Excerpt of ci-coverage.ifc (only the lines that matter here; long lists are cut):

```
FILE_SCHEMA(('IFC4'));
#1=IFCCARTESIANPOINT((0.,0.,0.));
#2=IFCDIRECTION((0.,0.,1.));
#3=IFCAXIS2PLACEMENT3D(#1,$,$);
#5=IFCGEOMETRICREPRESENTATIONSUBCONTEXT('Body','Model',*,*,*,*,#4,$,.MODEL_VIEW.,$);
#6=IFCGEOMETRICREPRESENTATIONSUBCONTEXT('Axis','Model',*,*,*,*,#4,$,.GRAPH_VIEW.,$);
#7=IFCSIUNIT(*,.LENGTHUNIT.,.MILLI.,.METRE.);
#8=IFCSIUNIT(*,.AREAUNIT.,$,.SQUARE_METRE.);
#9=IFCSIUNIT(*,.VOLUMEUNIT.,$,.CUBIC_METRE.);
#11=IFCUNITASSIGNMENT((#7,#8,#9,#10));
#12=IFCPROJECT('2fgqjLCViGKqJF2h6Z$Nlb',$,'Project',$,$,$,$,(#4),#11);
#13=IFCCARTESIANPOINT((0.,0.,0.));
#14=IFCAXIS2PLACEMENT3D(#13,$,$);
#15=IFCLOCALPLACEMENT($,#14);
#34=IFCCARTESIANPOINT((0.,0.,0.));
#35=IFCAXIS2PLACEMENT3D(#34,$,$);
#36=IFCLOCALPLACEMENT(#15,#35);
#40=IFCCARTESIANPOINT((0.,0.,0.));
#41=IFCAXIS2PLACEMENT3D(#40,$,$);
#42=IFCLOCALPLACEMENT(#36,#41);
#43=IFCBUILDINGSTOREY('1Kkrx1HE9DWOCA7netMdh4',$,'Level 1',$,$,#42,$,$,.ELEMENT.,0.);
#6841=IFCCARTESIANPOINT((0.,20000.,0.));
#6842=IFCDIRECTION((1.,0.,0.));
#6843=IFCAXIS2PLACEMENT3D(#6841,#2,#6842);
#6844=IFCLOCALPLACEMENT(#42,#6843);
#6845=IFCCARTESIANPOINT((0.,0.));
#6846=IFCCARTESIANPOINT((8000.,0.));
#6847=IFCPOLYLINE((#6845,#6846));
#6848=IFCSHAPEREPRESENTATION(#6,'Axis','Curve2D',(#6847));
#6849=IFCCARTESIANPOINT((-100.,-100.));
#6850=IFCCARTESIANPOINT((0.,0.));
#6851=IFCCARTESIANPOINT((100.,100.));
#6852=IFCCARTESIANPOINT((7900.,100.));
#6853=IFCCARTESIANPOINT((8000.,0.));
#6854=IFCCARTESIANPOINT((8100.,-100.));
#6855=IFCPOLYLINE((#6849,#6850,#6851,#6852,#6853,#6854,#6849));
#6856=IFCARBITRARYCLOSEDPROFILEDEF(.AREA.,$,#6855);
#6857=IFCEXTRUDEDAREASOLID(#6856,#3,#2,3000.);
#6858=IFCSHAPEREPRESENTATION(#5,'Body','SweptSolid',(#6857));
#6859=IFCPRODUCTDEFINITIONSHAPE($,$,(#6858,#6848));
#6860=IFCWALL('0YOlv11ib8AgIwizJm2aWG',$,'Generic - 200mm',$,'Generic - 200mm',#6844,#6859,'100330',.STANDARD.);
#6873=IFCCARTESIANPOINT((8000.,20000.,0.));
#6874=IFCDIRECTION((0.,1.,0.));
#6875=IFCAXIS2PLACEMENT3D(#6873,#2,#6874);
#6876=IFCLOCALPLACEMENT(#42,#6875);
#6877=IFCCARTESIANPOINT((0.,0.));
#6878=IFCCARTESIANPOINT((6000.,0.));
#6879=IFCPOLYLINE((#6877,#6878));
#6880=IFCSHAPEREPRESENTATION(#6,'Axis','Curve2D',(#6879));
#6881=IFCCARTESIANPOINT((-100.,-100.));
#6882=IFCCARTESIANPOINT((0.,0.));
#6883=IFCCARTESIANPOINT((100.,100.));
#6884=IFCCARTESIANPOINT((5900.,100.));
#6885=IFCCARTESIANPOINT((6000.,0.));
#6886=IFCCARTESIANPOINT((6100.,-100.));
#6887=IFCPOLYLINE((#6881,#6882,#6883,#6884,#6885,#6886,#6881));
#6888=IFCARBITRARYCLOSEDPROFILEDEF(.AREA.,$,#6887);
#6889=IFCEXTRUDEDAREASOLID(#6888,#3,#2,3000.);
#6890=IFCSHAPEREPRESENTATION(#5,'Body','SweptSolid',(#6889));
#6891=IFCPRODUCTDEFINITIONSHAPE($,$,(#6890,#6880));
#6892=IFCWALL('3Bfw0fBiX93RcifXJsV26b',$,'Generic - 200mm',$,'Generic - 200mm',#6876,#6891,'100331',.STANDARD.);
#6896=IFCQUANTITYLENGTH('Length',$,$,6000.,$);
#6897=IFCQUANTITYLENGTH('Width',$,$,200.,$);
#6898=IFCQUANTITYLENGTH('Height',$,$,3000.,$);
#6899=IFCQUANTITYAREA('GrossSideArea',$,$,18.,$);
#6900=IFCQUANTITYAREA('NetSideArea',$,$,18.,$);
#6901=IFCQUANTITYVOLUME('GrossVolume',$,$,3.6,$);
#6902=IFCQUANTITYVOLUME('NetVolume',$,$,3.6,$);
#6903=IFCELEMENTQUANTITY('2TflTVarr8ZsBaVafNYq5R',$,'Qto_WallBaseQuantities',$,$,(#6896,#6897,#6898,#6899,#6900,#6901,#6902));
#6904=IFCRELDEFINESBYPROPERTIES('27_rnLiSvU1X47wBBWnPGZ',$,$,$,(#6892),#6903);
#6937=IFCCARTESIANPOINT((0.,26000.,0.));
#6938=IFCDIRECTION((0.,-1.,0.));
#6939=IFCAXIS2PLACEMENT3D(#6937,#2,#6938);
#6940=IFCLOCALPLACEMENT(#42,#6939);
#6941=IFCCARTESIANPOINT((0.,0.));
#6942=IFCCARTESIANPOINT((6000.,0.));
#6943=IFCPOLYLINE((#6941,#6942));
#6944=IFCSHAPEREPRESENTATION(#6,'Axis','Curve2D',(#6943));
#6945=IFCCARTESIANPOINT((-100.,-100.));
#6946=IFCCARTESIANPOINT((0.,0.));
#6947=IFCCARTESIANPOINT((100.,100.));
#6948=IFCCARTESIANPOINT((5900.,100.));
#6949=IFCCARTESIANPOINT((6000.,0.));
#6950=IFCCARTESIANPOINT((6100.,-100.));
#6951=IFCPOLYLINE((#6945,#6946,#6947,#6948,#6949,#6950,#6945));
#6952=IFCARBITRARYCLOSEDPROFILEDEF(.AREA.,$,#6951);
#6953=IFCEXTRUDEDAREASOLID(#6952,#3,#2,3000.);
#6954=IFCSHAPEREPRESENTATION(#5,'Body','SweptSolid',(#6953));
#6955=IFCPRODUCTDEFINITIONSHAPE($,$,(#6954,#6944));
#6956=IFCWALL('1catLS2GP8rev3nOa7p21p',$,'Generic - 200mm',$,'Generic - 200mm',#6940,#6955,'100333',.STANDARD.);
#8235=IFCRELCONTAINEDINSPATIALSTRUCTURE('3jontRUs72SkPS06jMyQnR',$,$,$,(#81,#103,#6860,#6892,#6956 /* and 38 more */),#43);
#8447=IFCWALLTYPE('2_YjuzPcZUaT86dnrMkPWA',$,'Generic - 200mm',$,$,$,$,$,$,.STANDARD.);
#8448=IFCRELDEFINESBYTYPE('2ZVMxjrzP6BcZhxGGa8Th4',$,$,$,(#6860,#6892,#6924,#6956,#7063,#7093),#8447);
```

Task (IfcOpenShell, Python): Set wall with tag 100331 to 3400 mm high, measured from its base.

```python
import ifcopenshell
import ifcopenshell.api.pset
import ifcopenshell.geom
import ifcopenshell.util.element
import ifcopenshell.util.representation
import ifcopenshell.util.shape
import ifcopenshell.util.unit

model = ifcopenshell.open("ci-coverage.ifc")
unit_scale = ifcopenshell.util.unit.calculate_unit_scale(model)
area_scale = ifcopenshell.util.unit.calculate_unit_scale(model, "AREAUNIT")
volume_scale = ifcopenshell.util.unit.calculate_unit_scale(model, "VOLUMEUNIT")
settings = ifcopenshell.geom.settings()


def volume(element):
    """Net volume in cubic metres, openings subtracted."""
    shape = ifcopenshell.geom.create_shape(settings, element)
    return ifcopenshell.util.shape.get_volume(shape.geometry)


wall = model.by_guid("3Bfw0fBiX93RcifXJsV26b")
before = volume(wall)

body = ifcopenshell.util.representation.get_representation(wall, "Model", "Body")
solid = body.Items[0]
old_height = solid.Depth
solid.Depth = 3.4 / unit_scale
after = volume(wall)
thickness = 0.2  # wall thickness in metres

# Update the stored height, areas and volumes.
qto = model.by_id(ifcopenshell.util.element.get_pset(wall, "Qto_WallBaseQuantities", should_inherit=False)["id"])
ifcopenshell.api.pset.edit_qto(model, qto=qto, properties={
    "Height": solid.Depth,
    "GrossSideArea": ifcopenshell.util.element.get_pset(wall, "Qto_WallBaseQuantities", "GrossSideArea") * solid.Depth / old_height,
    "NetSideArea": after / thickness / area_scale,
    "GrossVolume": ifcopenshell.util.element.get_pset(wall, "Qto_WallBaseQuantities", "GrossVolume") * solid.Depth / old_height,
    "NetVolume": after / volume_scale,
})

print(f"height {old_height:g} -> {solid.Depth:g}, volume {before:.3f} -> {after:.3f} m3")

model.write("ci-coverage_rev.ifc")
```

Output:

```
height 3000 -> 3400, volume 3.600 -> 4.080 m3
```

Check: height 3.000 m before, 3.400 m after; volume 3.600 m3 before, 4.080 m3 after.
